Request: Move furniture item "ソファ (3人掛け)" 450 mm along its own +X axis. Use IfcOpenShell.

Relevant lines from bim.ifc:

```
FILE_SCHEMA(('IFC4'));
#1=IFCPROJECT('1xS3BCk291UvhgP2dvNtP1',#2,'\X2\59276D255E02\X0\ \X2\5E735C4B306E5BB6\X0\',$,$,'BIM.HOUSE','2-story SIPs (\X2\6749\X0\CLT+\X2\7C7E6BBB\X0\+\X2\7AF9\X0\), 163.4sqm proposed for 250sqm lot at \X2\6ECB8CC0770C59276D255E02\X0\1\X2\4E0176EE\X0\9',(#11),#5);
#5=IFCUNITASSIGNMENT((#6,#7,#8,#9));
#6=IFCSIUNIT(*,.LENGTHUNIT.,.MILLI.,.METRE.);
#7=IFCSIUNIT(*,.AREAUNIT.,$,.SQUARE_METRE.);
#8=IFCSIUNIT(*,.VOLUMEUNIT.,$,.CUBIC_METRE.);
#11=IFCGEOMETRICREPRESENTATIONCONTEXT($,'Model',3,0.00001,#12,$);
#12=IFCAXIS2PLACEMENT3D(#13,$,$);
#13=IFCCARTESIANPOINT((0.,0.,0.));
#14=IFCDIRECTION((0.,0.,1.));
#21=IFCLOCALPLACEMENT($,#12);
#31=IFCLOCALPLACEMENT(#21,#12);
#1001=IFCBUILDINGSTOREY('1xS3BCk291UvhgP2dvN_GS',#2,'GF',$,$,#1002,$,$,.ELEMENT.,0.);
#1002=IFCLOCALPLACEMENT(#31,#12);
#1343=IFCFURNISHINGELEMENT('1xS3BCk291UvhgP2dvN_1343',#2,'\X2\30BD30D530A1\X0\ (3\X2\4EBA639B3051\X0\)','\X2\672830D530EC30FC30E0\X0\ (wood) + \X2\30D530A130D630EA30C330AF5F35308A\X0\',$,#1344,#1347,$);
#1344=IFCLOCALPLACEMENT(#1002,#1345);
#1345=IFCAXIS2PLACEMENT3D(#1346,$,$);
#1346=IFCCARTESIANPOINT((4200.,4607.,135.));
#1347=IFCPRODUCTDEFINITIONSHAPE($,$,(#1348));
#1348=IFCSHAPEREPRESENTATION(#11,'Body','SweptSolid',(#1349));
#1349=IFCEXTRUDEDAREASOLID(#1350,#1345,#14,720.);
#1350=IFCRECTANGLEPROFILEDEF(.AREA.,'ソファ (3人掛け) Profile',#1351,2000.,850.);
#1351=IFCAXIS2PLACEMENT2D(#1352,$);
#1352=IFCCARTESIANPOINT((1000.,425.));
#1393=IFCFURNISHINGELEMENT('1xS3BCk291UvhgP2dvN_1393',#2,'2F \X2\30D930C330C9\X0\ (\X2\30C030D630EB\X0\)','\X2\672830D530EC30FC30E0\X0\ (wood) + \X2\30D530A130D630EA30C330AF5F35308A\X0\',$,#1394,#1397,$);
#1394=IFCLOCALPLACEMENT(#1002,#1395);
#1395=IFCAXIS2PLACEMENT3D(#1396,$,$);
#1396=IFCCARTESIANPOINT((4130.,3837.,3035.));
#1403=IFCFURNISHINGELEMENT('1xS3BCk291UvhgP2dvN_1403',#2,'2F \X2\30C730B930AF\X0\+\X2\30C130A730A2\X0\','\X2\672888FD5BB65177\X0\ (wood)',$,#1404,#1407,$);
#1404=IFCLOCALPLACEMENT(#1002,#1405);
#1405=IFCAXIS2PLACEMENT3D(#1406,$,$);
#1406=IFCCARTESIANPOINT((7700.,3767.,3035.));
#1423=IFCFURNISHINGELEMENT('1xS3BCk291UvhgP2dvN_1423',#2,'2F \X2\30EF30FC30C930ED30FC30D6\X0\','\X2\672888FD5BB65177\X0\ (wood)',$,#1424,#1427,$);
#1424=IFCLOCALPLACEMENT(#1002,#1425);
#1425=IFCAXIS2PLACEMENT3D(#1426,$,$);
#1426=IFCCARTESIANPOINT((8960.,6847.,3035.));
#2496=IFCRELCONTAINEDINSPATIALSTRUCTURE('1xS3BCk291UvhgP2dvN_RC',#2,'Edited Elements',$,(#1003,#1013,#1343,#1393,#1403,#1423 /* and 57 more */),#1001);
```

```python
import ifcopenshell
import ifcopenshell.api.geometry
import ifcopenshell.util.placement
import ifcopenshell.util.unit

model = ifcopenshell.open("bim.ifc")
unit_scale = ifcopenshell.util.unit.calculate_unit_scale(model)

item = model.by_guid("1xS3BCk291UvhgP2dvN_1343")
matrix = ifcopenshell.util.placement.get_local_placement(item.ObjectPlacement)
matrix[:3, 3] += matrix[:3, 0] * 0.45 / unit_scale
ifcopenshell.api.geometry.edit_object_placement(model, product=item, matrix=matrix, is_si=False)

print(ifcopenshell.util.placement.get_local_placement(item.ObjectPlacement).round(3) + 0.0)

model.write("bim_updated.ifc")
```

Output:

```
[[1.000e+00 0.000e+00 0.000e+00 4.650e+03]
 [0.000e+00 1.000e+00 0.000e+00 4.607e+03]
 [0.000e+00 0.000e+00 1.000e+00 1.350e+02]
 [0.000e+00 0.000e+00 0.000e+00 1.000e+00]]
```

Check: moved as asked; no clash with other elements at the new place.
